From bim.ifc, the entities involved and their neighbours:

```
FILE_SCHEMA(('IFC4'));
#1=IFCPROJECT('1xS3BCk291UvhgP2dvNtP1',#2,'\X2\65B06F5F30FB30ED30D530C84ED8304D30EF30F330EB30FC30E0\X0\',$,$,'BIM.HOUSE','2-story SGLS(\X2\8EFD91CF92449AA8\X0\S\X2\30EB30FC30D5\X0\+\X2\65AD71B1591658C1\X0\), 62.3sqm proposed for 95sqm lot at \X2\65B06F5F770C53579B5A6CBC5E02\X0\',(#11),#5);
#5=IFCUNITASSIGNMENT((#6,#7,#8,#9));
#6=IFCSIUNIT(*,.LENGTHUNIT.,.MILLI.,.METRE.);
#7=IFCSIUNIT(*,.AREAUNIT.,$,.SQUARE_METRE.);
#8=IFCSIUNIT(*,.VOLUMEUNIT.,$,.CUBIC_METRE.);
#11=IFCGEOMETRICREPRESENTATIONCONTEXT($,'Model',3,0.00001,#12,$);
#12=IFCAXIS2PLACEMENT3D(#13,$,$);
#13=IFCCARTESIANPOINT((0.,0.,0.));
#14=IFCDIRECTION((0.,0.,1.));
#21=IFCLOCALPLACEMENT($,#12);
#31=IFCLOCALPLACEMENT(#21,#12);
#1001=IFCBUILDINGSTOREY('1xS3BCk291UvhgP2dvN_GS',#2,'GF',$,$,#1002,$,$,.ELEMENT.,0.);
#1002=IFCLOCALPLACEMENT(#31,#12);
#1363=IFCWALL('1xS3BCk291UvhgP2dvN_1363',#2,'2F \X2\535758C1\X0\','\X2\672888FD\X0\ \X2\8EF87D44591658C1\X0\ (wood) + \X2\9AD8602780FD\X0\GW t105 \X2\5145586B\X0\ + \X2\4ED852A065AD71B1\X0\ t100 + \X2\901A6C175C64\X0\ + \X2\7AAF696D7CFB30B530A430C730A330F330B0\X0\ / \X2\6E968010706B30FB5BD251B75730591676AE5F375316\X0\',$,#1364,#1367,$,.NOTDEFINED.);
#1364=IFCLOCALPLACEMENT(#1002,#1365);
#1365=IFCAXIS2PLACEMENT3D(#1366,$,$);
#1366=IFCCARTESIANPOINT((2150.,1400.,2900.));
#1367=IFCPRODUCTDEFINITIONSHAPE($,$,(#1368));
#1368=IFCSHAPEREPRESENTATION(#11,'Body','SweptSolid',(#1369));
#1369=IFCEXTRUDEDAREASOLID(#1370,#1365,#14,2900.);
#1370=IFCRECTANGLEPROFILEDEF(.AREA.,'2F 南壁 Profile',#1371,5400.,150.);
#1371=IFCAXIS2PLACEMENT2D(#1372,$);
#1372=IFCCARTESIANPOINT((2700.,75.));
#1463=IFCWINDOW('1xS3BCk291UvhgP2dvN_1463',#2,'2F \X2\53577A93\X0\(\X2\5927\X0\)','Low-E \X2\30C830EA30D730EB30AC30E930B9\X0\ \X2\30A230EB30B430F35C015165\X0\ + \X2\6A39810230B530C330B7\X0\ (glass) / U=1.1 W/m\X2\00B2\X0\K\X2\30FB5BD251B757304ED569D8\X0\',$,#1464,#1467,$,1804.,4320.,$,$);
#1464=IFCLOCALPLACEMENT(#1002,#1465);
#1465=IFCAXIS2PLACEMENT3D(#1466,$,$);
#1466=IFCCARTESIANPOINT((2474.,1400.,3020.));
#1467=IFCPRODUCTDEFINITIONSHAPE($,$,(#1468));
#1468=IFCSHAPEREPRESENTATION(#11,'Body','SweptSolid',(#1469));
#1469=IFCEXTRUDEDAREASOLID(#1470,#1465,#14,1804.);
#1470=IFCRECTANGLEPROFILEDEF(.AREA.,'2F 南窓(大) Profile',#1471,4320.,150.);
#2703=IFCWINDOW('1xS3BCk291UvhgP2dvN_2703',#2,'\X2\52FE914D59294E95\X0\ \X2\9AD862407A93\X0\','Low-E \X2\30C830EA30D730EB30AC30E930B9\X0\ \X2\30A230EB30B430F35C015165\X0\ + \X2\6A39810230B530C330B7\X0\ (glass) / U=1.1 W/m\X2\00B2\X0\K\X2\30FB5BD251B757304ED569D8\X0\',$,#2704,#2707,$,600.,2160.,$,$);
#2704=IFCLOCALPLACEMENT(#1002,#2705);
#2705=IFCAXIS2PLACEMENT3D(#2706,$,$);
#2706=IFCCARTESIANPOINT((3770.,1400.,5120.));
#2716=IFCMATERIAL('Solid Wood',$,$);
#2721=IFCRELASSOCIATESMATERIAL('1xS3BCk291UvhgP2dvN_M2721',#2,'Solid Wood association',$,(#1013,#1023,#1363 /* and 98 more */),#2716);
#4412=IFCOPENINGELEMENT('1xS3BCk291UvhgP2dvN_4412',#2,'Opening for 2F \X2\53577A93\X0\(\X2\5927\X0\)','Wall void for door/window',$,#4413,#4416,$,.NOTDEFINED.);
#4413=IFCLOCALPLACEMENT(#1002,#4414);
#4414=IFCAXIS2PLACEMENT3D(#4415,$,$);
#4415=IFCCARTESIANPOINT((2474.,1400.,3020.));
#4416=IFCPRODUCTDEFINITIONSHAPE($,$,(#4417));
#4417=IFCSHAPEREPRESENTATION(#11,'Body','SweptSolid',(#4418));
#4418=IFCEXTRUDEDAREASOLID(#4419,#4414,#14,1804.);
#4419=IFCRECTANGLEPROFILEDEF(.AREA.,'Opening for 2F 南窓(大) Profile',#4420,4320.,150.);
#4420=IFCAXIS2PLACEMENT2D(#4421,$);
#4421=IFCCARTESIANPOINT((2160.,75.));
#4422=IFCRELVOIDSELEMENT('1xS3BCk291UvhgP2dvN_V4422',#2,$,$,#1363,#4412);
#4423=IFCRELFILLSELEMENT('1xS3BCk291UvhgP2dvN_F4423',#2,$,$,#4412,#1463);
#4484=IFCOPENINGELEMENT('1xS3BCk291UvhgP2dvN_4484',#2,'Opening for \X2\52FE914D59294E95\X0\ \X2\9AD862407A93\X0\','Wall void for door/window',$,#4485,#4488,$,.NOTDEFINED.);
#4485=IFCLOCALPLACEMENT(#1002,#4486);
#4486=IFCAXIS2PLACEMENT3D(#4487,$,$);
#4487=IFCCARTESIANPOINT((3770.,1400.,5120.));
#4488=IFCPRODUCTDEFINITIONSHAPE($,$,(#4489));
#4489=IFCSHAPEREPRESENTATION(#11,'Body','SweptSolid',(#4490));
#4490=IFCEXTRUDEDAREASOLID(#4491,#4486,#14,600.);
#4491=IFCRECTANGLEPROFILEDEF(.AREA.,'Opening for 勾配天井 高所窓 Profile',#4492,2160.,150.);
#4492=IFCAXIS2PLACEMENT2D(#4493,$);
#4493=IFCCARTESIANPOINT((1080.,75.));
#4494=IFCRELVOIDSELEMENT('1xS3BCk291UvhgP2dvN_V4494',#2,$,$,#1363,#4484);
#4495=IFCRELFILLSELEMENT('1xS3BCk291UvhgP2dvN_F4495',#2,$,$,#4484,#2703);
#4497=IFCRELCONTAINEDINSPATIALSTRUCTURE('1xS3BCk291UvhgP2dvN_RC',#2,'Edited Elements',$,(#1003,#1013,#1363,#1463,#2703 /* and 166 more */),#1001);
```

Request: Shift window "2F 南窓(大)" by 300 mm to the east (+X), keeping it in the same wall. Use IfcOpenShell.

```python
import ifcopenshell
import ifcopenshell.api.geometry
import ifcopenshell.util.placement
import ifcopenshell.util.unit

model = ifcopenshell.open("bim.ifc")
unit_scale = ifcopenshell.util.unit.calculate_unit_scale(model)

window = model.by_guid("1xS3BCk291UvhgP2dvN_1463")
opening = window.FillsVoids[0].RelatingOpeningElement
wall = opening.VoidsElements[0].RelatingBuildingElement

wall_matrix = ifcopenshell.util.placement.get_local_placement(wall.ObjectPlacement)
shift = wall_matrix[:3, 0] * 0.3 / unit_scale
before = ifcopenshell.util.placement.get_local_placement(window.ObjectPlacement)[:3, 3].copy()

# The window is not placed relative to its opening, so move both.
for product in (opening, window):
    matrix = ifcopenshell.util.placement.get_local_placement(product.ObjectPlacement)
    matrix[:3, 3] += shift
    ifcopenshell.api.geometry.edit_object_placement(model, product=product, matrix=matrix, is_si=False)

after = ifcopenshell.util.placement.get_local_placement(window.ObjectPlacement)[:3, 3]
print("window moved by", (after - before).round(3) + 0.0)

model.write("bim_rev.ifc")
```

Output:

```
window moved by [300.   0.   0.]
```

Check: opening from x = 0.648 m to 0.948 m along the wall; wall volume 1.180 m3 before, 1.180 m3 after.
